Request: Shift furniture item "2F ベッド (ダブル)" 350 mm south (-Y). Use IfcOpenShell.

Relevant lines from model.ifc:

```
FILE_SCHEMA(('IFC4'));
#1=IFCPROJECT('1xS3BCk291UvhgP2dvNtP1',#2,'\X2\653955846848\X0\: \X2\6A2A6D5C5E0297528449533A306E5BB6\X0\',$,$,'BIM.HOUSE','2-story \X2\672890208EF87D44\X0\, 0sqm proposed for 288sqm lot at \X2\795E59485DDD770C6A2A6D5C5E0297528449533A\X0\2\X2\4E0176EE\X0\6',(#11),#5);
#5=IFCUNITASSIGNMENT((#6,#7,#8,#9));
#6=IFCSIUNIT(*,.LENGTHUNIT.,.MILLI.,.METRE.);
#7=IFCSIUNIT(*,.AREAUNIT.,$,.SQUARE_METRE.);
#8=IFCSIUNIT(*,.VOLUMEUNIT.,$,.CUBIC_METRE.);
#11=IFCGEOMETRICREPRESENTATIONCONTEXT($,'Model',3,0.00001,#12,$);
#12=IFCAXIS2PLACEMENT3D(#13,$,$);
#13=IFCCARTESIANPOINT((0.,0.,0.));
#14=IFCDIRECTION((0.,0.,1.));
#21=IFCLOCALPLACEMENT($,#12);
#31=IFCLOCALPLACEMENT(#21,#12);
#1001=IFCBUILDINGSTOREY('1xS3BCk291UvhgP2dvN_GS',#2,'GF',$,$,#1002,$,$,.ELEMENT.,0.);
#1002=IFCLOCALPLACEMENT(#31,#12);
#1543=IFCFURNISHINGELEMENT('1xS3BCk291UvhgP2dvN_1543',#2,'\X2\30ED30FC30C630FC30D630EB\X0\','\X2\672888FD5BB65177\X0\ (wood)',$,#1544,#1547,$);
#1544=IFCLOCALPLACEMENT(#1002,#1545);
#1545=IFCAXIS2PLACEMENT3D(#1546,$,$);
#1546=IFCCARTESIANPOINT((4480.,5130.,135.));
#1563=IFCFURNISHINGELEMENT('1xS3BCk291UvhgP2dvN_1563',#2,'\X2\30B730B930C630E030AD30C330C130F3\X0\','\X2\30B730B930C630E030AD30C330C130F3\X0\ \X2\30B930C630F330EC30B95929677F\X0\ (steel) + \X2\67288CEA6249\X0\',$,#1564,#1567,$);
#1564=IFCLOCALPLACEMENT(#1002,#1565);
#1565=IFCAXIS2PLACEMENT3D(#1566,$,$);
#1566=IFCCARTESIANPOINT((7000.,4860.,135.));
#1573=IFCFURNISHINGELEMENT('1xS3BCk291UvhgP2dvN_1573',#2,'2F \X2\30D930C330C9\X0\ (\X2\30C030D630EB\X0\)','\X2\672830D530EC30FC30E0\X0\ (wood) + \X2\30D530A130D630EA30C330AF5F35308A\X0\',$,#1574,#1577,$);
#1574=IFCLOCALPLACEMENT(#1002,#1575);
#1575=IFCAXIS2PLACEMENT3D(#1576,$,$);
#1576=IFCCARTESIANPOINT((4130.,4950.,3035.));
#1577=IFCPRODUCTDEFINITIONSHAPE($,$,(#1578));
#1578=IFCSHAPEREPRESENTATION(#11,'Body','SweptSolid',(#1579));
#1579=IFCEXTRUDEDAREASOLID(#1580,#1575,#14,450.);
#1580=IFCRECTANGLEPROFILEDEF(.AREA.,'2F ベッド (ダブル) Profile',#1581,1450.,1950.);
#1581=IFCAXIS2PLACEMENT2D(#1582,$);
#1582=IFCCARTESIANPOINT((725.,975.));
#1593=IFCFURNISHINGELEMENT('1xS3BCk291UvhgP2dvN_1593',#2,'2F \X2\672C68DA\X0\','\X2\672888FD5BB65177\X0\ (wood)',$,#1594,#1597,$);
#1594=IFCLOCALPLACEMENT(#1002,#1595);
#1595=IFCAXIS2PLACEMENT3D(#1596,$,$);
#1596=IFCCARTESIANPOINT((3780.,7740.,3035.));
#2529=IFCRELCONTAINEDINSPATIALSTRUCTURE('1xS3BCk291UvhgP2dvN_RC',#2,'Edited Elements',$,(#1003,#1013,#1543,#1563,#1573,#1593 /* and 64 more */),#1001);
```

```python
import ifcopenshell
import ifcopenshell.api.geometry
import ifcopenshell.util.placement

model = ifcopenshell.open("model.ifc")

item = model.by_id(1573)
matrix = ifcopenshell.util.placement.get_local_placement(item.ObjectPlacement)
matrix[1, 3] -= 350.0
ifcopenshell.api.geometry.edit_object_placement(model, product=item, matrix=matrix, is_si=False)

print(ifcopenshell.util.placement.get_local_placement(item.ObjectPlacement).round(3) + 0.0)

model.write("model_edited.ifc")
```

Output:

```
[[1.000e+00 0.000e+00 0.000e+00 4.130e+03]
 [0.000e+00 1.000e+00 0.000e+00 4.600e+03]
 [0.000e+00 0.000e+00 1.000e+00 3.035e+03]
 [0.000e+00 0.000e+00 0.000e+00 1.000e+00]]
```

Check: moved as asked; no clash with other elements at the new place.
